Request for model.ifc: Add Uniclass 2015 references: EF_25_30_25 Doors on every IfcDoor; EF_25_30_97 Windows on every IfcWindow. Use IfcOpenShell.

First a look at what the model holds.

```python
import ifcopenshell

model = ifcopenshell.open("model.ifc")
print(model.schema)
print("classifications:", [c.Name for c in model.by_type("IfcClassification")])
for ifc_class in ("IfcDoor", "IfcRoof", "IfcStair", "IfcWall", "IfcWindow"):
    print(ifc_class, len(model.by_type(ifc_class)))
```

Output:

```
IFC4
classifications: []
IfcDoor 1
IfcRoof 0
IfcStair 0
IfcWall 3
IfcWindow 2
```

```python
import ifcopenshell
import ifcopenshell.api.classification

model = ifcopenshell.open("model.ifc")

system = ifcopenshell.api.classification.add_classification(model, classification="Uniclass 2015")

codes = {
    "IfcDoor": ("EF_25_30_25", "Doors"),
    "IfcWindow": ("EF_25_30_97", "Windows"),
}
for ifc_class, (code, name) in codes.items():
    products = model.by_type(ifc_class)
    ifcopenshell.api.classification.add_reference(
        model, products=products, classification=system, identification=code, name=name
    )
    print(code, len(products))

model.write("model_rev.ifc")
```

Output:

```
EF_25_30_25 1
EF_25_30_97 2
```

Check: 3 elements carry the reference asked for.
